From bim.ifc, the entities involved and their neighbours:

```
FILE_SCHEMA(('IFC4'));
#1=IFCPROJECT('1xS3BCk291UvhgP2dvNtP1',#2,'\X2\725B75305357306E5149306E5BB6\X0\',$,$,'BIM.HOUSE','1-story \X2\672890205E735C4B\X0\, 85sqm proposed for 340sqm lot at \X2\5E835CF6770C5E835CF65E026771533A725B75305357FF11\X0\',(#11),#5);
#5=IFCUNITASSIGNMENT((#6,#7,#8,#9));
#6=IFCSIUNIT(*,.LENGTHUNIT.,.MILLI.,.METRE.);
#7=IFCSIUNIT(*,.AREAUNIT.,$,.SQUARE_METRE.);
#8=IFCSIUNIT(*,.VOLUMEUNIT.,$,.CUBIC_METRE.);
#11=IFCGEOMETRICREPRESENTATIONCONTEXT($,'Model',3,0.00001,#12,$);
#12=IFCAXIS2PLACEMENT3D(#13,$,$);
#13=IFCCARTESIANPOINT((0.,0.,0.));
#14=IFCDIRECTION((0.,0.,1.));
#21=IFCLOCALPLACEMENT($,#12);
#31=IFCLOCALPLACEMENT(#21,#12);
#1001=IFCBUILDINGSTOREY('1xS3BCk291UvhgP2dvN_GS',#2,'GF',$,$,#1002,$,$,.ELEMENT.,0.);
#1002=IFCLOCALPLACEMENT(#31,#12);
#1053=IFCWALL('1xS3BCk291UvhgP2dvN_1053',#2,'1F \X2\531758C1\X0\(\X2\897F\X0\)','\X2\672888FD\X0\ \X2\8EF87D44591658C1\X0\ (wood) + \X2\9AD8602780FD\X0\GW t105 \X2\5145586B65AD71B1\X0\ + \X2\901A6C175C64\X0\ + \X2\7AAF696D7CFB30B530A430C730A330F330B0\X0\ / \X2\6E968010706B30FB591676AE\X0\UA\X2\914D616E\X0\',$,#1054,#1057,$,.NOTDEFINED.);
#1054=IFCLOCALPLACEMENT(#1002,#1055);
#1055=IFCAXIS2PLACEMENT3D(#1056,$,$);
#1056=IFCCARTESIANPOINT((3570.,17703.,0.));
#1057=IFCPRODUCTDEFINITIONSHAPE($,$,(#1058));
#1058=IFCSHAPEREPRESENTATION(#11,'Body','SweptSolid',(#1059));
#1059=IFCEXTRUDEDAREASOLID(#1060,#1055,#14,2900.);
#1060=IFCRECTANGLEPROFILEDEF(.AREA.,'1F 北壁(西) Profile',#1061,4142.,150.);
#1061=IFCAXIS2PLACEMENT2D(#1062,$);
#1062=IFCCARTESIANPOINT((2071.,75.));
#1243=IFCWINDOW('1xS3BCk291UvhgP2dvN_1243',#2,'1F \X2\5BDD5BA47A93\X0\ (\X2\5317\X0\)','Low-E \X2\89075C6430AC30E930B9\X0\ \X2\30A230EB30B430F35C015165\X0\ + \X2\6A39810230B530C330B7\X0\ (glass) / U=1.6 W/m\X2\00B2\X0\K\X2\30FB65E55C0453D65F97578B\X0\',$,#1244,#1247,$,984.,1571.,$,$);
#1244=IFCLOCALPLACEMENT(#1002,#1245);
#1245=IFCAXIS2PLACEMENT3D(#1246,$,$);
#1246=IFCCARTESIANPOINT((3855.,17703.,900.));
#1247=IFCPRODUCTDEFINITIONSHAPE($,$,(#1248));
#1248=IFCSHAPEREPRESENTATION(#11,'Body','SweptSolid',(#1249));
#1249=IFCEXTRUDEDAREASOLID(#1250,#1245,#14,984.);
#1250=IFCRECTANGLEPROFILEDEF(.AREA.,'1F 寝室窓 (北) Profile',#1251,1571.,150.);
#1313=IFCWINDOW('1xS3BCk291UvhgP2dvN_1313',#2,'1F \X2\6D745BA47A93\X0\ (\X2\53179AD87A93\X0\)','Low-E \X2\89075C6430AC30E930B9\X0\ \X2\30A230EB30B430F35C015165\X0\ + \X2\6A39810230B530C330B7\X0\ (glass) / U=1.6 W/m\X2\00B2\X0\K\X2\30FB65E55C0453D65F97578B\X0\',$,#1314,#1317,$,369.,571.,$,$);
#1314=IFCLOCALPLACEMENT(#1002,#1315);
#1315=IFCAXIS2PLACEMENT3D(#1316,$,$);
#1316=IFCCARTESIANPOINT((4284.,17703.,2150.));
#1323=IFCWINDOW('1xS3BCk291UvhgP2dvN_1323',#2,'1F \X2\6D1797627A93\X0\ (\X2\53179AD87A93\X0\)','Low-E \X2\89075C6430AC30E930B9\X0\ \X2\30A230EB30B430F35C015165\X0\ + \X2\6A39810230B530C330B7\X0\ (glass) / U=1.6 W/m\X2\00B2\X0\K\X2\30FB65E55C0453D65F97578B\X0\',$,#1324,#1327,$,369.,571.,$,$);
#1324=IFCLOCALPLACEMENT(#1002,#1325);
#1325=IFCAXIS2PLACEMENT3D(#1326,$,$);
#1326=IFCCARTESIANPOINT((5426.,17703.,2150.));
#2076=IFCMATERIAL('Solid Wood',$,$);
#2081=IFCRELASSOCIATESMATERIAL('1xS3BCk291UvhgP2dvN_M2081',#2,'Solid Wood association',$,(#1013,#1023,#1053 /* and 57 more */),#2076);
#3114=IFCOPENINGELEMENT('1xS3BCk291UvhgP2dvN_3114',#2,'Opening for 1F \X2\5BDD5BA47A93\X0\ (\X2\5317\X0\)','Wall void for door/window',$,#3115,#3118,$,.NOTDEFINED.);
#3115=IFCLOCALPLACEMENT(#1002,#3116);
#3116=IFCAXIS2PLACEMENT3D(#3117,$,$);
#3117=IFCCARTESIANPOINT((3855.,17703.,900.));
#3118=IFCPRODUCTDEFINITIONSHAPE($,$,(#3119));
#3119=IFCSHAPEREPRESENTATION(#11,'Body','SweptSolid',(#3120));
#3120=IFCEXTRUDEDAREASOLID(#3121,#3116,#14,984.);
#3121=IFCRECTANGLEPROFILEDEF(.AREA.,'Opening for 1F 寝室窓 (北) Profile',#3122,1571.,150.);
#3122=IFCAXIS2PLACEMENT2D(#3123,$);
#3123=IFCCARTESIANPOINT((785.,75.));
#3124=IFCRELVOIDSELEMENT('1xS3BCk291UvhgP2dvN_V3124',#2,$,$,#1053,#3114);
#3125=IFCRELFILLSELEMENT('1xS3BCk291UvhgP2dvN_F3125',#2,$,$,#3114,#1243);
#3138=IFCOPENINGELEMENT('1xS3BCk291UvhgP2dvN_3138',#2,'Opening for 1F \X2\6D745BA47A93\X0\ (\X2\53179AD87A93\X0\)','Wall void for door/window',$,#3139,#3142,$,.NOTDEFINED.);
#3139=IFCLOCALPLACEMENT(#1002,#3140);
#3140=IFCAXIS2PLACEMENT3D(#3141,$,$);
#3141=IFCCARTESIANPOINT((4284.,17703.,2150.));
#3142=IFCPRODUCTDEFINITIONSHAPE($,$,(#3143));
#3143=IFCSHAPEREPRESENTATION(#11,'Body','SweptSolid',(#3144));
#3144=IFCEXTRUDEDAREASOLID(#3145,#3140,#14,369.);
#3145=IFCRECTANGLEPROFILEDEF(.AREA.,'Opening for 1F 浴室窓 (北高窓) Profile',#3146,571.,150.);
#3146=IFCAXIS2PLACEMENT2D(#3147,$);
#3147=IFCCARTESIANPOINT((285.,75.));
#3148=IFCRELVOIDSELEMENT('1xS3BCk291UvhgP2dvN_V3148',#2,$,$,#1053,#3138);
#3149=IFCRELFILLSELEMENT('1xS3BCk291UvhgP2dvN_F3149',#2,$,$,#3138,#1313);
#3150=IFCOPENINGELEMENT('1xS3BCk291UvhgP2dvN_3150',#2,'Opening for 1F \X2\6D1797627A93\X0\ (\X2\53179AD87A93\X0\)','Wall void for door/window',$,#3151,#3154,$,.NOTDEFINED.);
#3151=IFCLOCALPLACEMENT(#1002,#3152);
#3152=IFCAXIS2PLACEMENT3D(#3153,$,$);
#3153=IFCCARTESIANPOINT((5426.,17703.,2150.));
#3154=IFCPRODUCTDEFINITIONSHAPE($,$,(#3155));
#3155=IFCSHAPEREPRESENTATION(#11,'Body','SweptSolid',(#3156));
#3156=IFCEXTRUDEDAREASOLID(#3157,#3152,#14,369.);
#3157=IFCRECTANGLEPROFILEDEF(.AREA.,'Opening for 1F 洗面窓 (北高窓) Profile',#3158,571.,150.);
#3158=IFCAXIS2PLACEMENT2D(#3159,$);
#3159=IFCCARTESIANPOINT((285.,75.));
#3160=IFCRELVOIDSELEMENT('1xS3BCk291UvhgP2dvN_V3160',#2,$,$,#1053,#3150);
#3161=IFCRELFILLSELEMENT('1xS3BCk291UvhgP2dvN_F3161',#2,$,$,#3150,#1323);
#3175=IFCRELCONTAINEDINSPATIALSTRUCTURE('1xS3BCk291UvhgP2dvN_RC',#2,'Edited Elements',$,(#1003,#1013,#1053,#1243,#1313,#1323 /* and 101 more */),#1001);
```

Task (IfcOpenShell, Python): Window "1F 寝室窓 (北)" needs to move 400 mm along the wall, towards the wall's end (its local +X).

```python
import ifcopenshell
import ifcopenshell.api.geometry
import ifcopenshell.util.placement
import ifcopenshell.util.unit

model = ifcopenshell.open("bim.ifc")
unit_scale = ifcopenshell.util.unit.calculate_unit_scale(model)

window = model.by_id(1243)
opening = window.FillsVoids[0].RelatingOpeningElement
wall = opening.VoidsElements[0].RelatingBuildingElement

wall_matrix = ifcopenshell.util.placement.get_local_placement(wall.ObjectPlacement)
shift = wall_matrix[:3, 0] * 0.4 / unit_scale
before = ifcopenshell.util.placement.get_local_placement(window.ObjectPlacement)[:3, 3].copy()

# The window is not placed relative to its opening, so move both.
for product in (opening, window):
    matrix = ifcopenshell.util.placement.get_local_placement(product.ObjectPlacement)
    matrix[:3, 3] += shift
    ifcopenshell.api.geometry.edit_object_placement(model, product=product, matrix=matrix, is_si=False)

after = ifcopenshell.util.placement.get_local_placement(window.ObjectPlacement)[:3, 3]
print("window moved by", (after - before).round(3) + 0.0)

model.write("bim_edited.ifc")
```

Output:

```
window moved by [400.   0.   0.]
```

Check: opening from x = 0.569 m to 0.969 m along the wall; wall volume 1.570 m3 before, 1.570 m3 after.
